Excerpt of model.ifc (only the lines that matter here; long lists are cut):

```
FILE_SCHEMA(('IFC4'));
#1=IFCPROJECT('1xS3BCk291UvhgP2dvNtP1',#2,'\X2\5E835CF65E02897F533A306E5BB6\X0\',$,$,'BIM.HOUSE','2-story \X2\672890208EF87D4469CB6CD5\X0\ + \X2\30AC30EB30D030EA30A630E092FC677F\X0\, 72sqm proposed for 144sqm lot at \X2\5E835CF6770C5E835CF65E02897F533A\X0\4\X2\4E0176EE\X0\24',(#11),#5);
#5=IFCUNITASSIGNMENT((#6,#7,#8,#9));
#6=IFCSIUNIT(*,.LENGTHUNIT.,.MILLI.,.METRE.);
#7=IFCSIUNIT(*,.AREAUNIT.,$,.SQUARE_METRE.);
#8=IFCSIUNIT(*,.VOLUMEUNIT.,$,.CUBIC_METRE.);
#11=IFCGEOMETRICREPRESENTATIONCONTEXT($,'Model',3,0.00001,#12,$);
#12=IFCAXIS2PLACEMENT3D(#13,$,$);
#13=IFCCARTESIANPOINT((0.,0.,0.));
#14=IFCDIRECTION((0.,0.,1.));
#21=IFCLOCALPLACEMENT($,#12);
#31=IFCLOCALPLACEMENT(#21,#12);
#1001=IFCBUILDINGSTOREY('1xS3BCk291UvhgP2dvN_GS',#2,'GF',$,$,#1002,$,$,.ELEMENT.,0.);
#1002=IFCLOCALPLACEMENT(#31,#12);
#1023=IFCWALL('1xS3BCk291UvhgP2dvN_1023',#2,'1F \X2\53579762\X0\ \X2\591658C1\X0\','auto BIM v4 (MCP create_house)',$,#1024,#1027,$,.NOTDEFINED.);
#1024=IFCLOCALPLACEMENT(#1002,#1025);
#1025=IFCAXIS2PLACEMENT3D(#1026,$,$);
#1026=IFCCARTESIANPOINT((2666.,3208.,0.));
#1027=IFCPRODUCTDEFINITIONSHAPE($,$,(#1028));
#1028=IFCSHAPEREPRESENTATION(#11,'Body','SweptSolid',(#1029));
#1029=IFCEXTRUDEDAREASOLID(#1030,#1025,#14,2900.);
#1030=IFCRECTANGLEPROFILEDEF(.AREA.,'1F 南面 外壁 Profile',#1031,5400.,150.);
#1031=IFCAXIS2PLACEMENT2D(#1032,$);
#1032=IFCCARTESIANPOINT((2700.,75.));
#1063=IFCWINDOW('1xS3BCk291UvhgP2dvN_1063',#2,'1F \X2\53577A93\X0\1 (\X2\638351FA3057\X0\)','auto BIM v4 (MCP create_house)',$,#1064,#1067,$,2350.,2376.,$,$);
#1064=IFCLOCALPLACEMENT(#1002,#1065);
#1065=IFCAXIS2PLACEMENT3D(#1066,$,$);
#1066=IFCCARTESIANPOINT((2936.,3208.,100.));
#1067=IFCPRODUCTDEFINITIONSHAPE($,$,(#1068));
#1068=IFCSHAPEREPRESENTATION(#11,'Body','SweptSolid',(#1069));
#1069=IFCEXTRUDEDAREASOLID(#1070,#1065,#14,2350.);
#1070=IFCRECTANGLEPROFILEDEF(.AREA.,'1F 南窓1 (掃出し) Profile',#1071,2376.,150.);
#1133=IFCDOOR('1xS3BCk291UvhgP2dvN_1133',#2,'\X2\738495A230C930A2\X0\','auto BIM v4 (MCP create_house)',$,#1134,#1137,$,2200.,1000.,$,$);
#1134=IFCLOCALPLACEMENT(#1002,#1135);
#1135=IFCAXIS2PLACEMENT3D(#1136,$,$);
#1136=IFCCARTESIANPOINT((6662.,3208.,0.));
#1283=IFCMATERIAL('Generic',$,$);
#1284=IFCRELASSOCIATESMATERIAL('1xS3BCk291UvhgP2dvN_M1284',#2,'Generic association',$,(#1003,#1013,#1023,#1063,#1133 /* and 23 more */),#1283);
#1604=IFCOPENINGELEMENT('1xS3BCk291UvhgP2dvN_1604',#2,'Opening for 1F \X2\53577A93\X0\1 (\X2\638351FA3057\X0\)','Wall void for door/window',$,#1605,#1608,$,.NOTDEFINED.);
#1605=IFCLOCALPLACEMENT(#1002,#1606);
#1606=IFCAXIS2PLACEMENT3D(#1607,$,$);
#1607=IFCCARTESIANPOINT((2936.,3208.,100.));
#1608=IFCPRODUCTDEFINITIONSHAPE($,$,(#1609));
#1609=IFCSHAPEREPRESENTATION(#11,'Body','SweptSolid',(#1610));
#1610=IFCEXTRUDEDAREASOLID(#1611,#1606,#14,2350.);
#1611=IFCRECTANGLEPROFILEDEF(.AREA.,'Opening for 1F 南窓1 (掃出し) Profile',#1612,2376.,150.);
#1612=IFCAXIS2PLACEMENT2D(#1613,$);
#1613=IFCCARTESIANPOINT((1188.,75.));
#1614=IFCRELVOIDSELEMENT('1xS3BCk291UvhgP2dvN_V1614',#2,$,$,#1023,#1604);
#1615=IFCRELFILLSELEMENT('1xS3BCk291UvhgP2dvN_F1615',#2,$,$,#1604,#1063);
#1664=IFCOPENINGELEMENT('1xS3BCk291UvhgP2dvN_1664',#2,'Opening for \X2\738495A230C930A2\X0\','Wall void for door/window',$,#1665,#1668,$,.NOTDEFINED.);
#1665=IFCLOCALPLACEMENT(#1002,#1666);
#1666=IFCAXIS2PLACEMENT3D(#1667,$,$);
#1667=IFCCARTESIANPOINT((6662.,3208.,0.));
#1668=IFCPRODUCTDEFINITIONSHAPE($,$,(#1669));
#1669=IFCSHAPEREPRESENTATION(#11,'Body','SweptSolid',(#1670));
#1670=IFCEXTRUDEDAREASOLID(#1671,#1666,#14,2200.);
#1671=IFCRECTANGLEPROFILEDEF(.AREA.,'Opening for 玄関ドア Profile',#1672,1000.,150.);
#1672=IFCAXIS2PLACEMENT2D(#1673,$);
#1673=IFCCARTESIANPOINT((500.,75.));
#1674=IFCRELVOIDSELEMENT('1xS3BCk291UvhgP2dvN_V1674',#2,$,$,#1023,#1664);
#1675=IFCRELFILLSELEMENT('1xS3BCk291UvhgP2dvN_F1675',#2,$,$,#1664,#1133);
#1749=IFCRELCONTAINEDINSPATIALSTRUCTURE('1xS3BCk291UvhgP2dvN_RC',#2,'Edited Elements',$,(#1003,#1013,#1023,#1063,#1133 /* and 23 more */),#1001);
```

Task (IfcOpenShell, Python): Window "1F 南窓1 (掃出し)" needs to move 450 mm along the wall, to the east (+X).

```python
import ifcopenshell
import ifcopenshell.api.geometry
import ifcopenshell.util.placement

model = ifcopenshell.open("model.ifc")

window = model.by_guid("1xS3BCk291UvhgP2dvN_1063")
opening = window.FillsVoids[0].RelatingOpeningElement
wall = opening.VoidsElements[0].RelatingBuildingElement

wall_matrix = ifcopenshell.util.placement.get_local_placement(wall.ObjectPlacement)
shift = wall_matrix[:3, 0] * 450.0
before = ifcopenshell.util.placement.get_local_placement(window.ObjectPlacement)[:3, 3].copy()

# The window is not placed relative to its opening, so move both.
for product in (opening, window):
    matrix = ifcopenshell.util.placement.get_local_placement(product.ObjectPlacement)
    matrix[:3, 3] += shift
    ifcopenshell.api.geometry.edit_object_placement(model, product=product, matrix=matrix, is_si=False)

after = ifcopenshell.util.placement.get_local_placement(window.ObjectPlacement)[:3, 3]
print("window moved by", (after - before).round(3) + 0.0)

model.write("model_rev.ifc")
```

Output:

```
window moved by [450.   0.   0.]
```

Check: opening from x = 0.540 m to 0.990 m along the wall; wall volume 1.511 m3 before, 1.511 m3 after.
